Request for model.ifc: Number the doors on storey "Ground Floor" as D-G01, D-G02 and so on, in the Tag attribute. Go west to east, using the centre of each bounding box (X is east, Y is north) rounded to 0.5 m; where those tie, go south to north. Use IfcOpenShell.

First a look at what the model holds.

```python
import ifcopenshell
import ifcopenshell.util.element
import ifcopenshell.util.placement

model = ifcopenshell.open("model.ifc")
print(model.schema)
storey = next(s for s in model.by_type("IfcBuildingStorey") if s.Name == "Ground Floor")
doors = [e for e in ifcopenshell.util.element.get_decomposition(storey) if e.is_a("IfcDoor")]
for e in sorted(doors, key=lambda e: e.id()):
    origin = ifcopenshell.util.placement.get_local_placement(e.ObjectPlacement)[:3, 3]
    print(e.id(), e.Tag, e.Name, origin.round(2) + 0.0, sep=" | ")
```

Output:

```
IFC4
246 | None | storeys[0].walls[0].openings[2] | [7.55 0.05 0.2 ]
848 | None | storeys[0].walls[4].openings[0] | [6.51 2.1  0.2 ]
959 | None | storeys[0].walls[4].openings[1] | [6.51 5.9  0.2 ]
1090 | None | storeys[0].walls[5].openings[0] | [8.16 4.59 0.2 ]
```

```python
import ifcopenshell
import ifcopenshell.geom
import ifcopenshell.util.element
import ifcopenshell.util.shape

model = ifcopenshell.open("model.ifc")
settings = ifcopenshell.geom.settings()
settings.set("use-world-coords", True)


def centre(element):
    shape = ifcopenshell.geom.create_shape(settings, element)
    return ifcopenshell.util.shape.get_bbox_centroid(shape.geometry)


storey = next(s for s in model.by_type("IfcBuildingStorey") if s.Name == "Ground Floor")
doors = [e for e in ifcopenshell.util.element.get_decomposition(storey) if e.is_a("IfcDoor")]

# Insertion points can sit at a corner or the storey origin, so sort by the geometry (in metres).
centres = {e: centre(e) for e in doors}
doors.sort(key=lambda e: (round(centres[e][0] / 0.5), centres[e][1]))

for i, e in enumerate(doors, start=1):
    number = f"D-G{i:02d}"
    e.Tag = number
    print(e.id(), number)

model.write("model_rev.ifc")
```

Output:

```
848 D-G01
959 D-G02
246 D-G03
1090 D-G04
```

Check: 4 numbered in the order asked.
